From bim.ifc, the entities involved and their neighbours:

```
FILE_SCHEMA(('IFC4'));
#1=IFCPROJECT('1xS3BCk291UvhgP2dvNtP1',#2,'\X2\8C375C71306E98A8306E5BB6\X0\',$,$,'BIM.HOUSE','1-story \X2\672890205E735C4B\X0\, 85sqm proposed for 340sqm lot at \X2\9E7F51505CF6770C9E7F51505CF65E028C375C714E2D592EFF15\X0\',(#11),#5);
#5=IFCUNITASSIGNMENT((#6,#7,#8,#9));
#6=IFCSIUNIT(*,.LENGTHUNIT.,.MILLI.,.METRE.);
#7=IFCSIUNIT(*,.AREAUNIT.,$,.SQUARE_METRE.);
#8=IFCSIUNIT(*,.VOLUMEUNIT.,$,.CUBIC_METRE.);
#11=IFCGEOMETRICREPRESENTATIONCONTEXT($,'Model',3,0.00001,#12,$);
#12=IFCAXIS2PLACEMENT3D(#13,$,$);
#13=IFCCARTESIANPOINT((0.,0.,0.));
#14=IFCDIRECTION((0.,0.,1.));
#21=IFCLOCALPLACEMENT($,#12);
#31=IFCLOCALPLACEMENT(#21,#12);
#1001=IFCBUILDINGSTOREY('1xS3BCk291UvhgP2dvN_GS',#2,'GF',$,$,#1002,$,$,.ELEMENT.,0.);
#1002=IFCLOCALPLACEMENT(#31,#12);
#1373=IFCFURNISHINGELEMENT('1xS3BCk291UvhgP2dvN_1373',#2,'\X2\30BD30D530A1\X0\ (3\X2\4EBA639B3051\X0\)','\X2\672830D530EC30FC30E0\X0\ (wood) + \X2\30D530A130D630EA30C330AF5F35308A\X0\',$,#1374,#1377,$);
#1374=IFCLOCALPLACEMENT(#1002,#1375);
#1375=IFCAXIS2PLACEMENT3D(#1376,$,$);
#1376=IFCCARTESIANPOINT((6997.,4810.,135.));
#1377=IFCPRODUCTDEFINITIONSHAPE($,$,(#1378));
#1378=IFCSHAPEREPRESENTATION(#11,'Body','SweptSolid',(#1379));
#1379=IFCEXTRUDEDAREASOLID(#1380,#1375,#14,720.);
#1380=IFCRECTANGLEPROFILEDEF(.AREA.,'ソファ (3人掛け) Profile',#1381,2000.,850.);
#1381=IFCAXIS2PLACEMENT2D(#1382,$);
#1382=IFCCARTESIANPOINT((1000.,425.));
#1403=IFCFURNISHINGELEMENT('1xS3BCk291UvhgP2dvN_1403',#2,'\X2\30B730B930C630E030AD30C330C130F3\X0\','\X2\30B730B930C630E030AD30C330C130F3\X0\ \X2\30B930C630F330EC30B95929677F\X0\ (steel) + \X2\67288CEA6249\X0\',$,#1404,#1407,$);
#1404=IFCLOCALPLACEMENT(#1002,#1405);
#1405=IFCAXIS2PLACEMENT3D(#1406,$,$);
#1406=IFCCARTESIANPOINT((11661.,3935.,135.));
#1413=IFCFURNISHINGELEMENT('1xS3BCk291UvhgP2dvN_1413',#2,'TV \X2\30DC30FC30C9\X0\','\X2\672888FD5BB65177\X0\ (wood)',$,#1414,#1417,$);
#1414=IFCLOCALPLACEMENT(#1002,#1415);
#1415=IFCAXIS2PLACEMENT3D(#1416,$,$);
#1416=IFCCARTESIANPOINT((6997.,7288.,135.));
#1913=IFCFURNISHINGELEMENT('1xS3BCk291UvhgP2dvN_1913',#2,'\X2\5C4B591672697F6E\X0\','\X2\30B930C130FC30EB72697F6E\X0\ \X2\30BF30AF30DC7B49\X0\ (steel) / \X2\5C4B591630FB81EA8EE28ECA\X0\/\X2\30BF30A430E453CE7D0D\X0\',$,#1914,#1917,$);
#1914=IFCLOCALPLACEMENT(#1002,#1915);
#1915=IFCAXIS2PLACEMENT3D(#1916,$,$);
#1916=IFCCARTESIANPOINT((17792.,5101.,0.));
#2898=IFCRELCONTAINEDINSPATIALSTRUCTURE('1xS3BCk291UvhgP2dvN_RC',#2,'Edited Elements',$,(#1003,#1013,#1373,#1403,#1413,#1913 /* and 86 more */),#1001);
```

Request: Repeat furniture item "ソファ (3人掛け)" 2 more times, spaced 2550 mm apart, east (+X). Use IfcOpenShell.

```python
import numpy as np
import ifcopenshell
import ifcopenshell.api.geometry
import ifcopenshell.api.root
import ifcopenshell.util.element
import ifcopenshell.util.placement
import ifcopenshell.util.unit

model = ifcopenshell.open("bim.ifc")
unit_scale = ifcopenshell.util.unit.calculate_unit_scale(model)


def reuse_history(source, copy):
    """copy_class also copies each property set's owner history, people and application; keep the originals."""
    for rel in copy.IsDefinedBy:
        if rel.is_a("IfcRelDefinesByProperties") and (history := rel.RelatingPropertyDefinition.OwnerHistory):
            rel.RelatingPropertyDefinition.OwnerHistory = source.OwnerHistory
            ifcopenshell.util.element.remove_deep2(model, history)


source = model.by_guid("1xS3BCk291UvhgP2dvN_1373")
base = ifcopenshell.util.placement.get_local_placement(source.ObjectPlacement)
step = np.array([1.0, 0.0, 0.0]) * 2.55 / unit_scale

for i in range(1, 3):
    copy = ifcopenshell.api.root.copy_class(model, product=source)
    copy.Representation = ifcopenshell.util.element.copy_deep(
        model, source.Representation, exclude=["IfcGeometricRepresentationContext", "IfcRepresentationMap"]
    )
    reuse_history(source, copy)
    matrix = base.copy()
    matrix[:3, 3] += i * step
    print("added at", matrix[:3, 3].round(3) + 0.0)
    ifcopenshell.api.geometry.edit_object_placement(model, product=copy, matrix=matrix, is_si=False)

model.write("bim_updated.ifc")
```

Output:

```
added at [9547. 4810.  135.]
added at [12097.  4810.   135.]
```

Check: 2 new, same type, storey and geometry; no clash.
